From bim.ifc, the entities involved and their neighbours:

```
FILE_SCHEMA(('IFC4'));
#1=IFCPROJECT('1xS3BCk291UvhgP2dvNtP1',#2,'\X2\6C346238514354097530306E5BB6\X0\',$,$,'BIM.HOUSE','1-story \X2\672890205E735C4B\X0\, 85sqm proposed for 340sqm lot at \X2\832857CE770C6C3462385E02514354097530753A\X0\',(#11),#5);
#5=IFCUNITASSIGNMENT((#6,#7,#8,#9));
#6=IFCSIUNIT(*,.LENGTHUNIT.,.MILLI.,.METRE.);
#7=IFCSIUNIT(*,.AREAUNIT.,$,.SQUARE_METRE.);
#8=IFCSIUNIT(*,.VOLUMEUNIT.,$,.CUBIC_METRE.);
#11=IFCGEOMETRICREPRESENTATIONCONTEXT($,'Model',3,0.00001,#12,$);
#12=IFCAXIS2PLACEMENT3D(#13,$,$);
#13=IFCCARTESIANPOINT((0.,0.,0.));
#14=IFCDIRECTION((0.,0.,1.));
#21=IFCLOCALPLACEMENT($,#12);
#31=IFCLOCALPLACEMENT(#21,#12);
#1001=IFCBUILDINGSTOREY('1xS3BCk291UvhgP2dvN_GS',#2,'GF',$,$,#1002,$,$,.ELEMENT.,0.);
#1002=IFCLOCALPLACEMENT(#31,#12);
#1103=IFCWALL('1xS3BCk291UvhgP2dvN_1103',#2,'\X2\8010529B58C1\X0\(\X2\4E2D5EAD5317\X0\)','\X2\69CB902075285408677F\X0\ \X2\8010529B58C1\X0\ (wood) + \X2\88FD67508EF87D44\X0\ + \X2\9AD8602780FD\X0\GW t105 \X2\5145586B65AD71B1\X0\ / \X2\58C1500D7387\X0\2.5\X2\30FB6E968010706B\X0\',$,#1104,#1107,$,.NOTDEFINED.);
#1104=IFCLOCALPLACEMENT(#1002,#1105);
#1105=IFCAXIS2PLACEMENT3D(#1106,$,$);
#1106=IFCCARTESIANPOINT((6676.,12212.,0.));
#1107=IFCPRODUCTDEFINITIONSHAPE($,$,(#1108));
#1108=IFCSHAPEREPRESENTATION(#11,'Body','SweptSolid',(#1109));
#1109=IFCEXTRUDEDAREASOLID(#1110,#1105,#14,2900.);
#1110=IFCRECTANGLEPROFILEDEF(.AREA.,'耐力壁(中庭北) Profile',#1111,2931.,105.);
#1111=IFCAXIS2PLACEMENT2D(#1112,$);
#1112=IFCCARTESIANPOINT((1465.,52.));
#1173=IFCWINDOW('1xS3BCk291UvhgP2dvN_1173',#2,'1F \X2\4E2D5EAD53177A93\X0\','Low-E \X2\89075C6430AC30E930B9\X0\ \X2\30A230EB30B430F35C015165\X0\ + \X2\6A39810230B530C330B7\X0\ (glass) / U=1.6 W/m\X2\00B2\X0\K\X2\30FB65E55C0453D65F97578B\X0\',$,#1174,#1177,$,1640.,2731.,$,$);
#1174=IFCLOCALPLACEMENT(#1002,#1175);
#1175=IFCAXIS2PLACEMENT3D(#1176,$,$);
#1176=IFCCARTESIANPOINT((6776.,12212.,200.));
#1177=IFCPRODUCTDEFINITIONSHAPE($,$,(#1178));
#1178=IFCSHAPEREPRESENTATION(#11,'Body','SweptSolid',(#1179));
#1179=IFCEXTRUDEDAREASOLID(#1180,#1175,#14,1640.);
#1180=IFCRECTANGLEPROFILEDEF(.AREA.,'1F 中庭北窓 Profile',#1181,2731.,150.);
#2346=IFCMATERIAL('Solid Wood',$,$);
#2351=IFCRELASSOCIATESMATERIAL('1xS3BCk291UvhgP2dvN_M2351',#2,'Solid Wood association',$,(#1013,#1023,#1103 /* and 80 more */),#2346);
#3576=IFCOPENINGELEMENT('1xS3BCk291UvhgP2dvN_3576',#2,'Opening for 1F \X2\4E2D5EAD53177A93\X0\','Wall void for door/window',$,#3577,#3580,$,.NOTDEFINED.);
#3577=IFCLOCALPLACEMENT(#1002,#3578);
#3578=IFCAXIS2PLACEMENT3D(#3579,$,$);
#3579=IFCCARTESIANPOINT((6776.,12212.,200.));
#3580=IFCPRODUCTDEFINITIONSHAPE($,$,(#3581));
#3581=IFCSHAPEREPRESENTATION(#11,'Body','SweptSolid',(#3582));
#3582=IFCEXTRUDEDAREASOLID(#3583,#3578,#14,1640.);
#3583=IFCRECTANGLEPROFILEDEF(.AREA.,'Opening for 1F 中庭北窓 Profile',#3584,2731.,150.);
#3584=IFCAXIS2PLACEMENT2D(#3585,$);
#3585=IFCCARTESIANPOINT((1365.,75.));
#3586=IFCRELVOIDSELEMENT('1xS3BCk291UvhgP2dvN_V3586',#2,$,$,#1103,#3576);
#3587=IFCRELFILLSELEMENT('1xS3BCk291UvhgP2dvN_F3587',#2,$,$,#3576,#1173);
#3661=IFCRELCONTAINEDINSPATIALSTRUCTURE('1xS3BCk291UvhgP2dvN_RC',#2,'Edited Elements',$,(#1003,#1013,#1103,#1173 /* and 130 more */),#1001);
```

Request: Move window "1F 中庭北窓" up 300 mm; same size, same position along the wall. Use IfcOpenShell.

```python
import numpy as np
import ifcopenshell
import ifcopenshell.api.geometry
import ifcopenshell.util.placement
import ifcopenshell.util.unit

model = ifcopenshell.open("bim.ifc")
unit_scale = ifcopenshell.util.unit.calculate_unit_scale(model)

window = model.by_guid("1xS3BCk291UvhgP2dvN_1173")
opening = window.FillsVoids[0].RelatingOpeningElement
dz = 0.3 / unit_scale

shift = np.array([0.0, 0.0, dz])
# The window is not placed relative to its opening, so move both.
for product in (opening, window):
    matrix = ifcopenshell.util.placement.get_local_placement(product.ObjectPlacement)
    matrix[:3, 3] += shift
    ifcopenshell.api.geometry.edit_object_placement(model, product=product, matrix=matrix, is_si=False)

print(f"moved by {dz * unit_scale:+.3f} m")

model.write("bim_rev.ifc")
```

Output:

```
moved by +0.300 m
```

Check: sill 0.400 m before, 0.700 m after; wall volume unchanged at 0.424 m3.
